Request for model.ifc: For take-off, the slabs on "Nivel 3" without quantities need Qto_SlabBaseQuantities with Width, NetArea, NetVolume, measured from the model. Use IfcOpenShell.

First a look at what the model holds.

```python
import ifcopenshell
import ifcopenshell.util.element
import ifcopenshell.util.unit

model = ifcopenshell.open("model.ifc")
print(model.schema)
for unit_type in ("LENGTHUNIT", "AREAUNIT", "VOLUMEUNIT"):
    print(unit_type, ifcopenshell.util.unit.calculate_unit_scale(model, unit_type))
storey = next(s for s in model.by_type("IfcBuildingStorey") if s.Name == "Nivel 3")
slabs = [e for e in ifcopenshell.util.element.get_decomposition(storey) if e.is_a("IfcSlab")]
for e in sorted(slabs, key=lambda e: e.id()):
    print(e.id(), e.is_a(), e.Name, list(ifcopenshell.util.element.get_psets(e, qtos_only=True)), sep=" | ")
```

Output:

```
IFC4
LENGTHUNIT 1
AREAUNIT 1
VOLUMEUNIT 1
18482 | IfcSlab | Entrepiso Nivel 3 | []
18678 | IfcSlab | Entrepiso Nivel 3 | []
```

```python
import ifcopenshell
import ifcopenshell.api.pset
import ifcopenshell.geom
import ifcopenshell.util.element
import ifcopenshell.util.shape
import ifcopenshell.util.unit

model = ifcopenshell.open("model.ifc")
unit_scale = ifcopenshell.util.unit.calculate_unit_scale(model)
area_scale = ifcopenshell.util.unit.calculate_unit_scale(model, "AREAUNIT")
volume_scale = ifcopenshell.util.unit.calculate_unit_scale(model, "VOLUMEUNIT")
settings = ifcopenshell.geom.settings()

storey = next(s for s in model.by_type("IfcBuildingStorey") if s.Name == "Nivel 3")
slabs = [e for e in ifcopenshell.util.element.get_decomposition(storey) if e.is_a("IfcSlab")]

for e in sorted(slabs, key=lambda e: e.id()):
    if ifcopenshell.util.element.get_psets(e, qtos_only=True, should_inherit=False):
        continue
    # Geometry comes back in metres, in the element's own axes.
    shape = ifcopenshell.geom.create_shape(settings, e)
    values = {
        "Width": ifcopenshell.util.shape.get_z(shape.geometry) / unit_scale,
        "NetArea": ifcopenshell.util.shape.get_footprint_area(shape.geometry) / area_scale,
        "NetVolume": ifcopenshell.util.shape.get_volume(shape.geometry) / volume_scale,
    }
    qto = ifcopenshell.api.pset.add_qto(model, product=e, name="Qto_SlabBaseQuantities")
    ifcopenshell.api.pset.edit_qto(model, qto=qto, properties=values)
    print(e.id(), {k: round(v, 3) for k, v in values.items()})

model.write("model_v2.ifc")
```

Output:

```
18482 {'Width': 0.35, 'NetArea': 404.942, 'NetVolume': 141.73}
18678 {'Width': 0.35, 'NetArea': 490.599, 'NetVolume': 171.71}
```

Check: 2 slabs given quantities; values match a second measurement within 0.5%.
